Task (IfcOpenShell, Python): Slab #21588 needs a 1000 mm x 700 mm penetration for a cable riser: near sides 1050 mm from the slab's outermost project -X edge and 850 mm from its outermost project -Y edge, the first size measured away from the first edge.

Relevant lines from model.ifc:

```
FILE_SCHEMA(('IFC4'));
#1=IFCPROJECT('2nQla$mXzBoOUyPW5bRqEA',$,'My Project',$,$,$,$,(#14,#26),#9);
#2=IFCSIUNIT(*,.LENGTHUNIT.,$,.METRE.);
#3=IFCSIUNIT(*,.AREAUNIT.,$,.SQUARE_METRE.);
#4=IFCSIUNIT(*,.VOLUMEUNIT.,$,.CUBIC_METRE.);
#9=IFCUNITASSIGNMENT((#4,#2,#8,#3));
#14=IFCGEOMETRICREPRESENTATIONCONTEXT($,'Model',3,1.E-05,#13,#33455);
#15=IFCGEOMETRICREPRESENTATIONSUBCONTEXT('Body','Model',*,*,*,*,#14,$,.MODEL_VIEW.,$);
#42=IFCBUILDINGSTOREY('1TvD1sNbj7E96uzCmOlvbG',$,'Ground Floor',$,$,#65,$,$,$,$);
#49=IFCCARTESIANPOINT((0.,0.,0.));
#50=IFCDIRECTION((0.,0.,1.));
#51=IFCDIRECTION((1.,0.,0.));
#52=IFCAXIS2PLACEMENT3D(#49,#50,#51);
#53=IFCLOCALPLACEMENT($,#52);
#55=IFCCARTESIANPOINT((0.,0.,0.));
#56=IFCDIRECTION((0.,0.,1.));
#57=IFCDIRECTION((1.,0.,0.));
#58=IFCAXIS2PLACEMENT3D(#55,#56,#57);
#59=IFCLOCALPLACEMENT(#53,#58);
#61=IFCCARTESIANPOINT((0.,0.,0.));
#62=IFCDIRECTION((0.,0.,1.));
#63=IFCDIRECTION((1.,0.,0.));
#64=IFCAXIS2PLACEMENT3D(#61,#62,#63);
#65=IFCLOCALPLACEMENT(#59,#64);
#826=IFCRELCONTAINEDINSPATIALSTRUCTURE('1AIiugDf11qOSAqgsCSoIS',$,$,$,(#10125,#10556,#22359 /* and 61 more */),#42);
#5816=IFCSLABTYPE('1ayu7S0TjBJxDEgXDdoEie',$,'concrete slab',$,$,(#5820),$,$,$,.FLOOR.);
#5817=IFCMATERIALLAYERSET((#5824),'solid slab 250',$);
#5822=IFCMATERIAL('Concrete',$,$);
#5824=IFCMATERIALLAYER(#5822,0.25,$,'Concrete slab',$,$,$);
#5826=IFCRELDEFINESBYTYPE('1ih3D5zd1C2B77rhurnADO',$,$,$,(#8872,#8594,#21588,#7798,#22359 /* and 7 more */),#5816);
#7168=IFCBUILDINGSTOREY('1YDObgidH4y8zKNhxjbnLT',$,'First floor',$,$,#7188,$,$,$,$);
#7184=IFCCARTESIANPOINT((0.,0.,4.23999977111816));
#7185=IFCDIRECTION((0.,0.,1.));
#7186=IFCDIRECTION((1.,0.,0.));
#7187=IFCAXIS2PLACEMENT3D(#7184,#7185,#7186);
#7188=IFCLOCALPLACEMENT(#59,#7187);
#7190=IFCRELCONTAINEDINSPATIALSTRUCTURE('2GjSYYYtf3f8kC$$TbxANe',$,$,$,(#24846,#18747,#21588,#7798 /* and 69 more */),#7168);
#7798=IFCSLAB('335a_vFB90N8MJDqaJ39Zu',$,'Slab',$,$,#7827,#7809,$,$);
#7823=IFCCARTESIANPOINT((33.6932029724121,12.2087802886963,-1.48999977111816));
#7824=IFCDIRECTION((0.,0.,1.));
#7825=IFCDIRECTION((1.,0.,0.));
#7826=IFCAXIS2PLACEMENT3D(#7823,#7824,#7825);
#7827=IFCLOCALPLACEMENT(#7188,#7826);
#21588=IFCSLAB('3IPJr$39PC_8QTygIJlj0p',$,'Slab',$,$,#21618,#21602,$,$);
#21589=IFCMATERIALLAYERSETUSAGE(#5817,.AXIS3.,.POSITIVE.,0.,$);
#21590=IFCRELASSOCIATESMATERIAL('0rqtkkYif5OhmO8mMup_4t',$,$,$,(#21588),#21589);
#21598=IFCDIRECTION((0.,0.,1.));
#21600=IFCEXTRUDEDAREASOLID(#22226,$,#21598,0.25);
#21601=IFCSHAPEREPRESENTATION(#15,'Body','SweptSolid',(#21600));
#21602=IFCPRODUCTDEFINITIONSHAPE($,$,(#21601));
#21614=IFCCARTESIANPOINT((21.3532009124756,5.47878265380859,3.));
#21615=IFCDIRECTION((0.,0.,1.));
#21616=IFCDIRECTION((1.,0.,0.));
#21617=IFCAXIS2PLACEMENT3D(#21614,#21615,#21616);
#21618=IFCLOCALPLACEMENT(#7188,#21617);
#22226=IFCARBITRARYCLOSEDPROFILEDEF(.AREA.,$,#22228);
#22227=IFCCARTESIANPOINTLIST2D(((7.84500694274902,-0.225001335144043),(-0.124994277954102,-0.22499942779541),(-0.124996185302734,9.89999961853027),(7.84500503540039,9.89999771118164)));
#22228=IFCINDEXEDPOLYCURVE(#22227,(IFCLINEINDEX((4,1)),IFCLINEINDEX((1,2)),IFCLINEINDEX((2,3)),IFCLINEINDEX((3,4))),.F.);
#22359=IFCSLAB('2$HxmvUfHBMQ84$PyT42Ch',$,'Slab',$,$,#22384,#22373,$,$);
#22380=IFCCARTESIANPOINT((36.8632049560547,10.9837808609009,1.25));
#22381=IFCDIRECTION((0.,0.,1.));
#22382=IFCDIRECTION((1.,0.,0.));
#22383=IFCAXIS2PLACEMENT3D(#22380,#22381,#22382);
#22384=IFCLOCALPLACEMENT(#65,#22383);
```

```python
import numpy as np
import ifcopenshell
import ifcopenshell.api.feature
import ifcopenshell.api.geometry
import ifcopenshell.api.root
import ifcopenshell.geom
import ifcopenshell.util.placement
import ifcopenshell.util.representation
import ifcopenshell.util.shape
import ifcopenshell.util.unit

model = ifcopenshell.open("model.ifc")
unit_scale = ifcopenshell.util.unit.calculate_unit_scale(model)
settings = ifcopenshell.geom.settings()


def volume(element):
    """Net volume in cubic metres, openings subtracted."""
    shape = ifcopenshell.geom.create_shape(settings, element)
    return ifcopenshell.util.shape.get_volume(shape.geometry)


slab = model.by_id(21588)
before = volume(slab)

# Extent in the slab's own axes, in metres. The edges named are its -X and -Y sides.
slab_shape = ifcopenshell.geom.create_shape(settings, slab)
vertices = ifcopenshell.util.shape.get_vertices(slab_shape.geometry)
x_min, y_min, bottom = vertices.min(axis=0)
top = vertices[:, 2].max()

opening = ifcopenshell.api.root.create_entity(model, ifc_class="IfcOpeningElement", name="Cable riser opening", predefined_type="OPENING")
context = ifcopenshell.util.representation.get_context(model, "Model", "Body", "MODEL_VIEW")
width, depth = 1, 0.7
outline = [(0.0, 0.0), (width, 0.0), (width, depth), (0.0, depth), (0.0, 0.0)]
# Overshoot both faces by 50 mm so the cut is clean.
shape = ifcopenshell.api.geometry.add_slab_representation(
    model, context=context, depth=top - bottom + 0.1, polyline=outline
)
ifcopenshell.api.geometry.assign_representation(model, product=opening, representation=shape)

matrix = ifcopenshell.util.placement.get_local_placement(slab.ObjectPlacement)
matrix[:, 3] = matrix @ np.append(np.array([x_min + 1.05, y_min + 0.85, bottom - 0.05]) / unit_scale, 1.0)
ifcopenshell.api.geometry.edit_object_placement(model, product=opening, matrix=matrix, is_si=False)
ifcopenshell.api.feature.add_feature(model, feature=opening, element=slab)

after = volume(slab)

print(f"slab volume {before:.3f} -> {after:.3f} m3")

model.write("model_updated.ifc")
```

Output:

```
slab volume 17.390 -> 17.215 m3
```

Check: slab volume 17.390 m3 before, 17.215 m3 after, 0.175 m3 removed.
